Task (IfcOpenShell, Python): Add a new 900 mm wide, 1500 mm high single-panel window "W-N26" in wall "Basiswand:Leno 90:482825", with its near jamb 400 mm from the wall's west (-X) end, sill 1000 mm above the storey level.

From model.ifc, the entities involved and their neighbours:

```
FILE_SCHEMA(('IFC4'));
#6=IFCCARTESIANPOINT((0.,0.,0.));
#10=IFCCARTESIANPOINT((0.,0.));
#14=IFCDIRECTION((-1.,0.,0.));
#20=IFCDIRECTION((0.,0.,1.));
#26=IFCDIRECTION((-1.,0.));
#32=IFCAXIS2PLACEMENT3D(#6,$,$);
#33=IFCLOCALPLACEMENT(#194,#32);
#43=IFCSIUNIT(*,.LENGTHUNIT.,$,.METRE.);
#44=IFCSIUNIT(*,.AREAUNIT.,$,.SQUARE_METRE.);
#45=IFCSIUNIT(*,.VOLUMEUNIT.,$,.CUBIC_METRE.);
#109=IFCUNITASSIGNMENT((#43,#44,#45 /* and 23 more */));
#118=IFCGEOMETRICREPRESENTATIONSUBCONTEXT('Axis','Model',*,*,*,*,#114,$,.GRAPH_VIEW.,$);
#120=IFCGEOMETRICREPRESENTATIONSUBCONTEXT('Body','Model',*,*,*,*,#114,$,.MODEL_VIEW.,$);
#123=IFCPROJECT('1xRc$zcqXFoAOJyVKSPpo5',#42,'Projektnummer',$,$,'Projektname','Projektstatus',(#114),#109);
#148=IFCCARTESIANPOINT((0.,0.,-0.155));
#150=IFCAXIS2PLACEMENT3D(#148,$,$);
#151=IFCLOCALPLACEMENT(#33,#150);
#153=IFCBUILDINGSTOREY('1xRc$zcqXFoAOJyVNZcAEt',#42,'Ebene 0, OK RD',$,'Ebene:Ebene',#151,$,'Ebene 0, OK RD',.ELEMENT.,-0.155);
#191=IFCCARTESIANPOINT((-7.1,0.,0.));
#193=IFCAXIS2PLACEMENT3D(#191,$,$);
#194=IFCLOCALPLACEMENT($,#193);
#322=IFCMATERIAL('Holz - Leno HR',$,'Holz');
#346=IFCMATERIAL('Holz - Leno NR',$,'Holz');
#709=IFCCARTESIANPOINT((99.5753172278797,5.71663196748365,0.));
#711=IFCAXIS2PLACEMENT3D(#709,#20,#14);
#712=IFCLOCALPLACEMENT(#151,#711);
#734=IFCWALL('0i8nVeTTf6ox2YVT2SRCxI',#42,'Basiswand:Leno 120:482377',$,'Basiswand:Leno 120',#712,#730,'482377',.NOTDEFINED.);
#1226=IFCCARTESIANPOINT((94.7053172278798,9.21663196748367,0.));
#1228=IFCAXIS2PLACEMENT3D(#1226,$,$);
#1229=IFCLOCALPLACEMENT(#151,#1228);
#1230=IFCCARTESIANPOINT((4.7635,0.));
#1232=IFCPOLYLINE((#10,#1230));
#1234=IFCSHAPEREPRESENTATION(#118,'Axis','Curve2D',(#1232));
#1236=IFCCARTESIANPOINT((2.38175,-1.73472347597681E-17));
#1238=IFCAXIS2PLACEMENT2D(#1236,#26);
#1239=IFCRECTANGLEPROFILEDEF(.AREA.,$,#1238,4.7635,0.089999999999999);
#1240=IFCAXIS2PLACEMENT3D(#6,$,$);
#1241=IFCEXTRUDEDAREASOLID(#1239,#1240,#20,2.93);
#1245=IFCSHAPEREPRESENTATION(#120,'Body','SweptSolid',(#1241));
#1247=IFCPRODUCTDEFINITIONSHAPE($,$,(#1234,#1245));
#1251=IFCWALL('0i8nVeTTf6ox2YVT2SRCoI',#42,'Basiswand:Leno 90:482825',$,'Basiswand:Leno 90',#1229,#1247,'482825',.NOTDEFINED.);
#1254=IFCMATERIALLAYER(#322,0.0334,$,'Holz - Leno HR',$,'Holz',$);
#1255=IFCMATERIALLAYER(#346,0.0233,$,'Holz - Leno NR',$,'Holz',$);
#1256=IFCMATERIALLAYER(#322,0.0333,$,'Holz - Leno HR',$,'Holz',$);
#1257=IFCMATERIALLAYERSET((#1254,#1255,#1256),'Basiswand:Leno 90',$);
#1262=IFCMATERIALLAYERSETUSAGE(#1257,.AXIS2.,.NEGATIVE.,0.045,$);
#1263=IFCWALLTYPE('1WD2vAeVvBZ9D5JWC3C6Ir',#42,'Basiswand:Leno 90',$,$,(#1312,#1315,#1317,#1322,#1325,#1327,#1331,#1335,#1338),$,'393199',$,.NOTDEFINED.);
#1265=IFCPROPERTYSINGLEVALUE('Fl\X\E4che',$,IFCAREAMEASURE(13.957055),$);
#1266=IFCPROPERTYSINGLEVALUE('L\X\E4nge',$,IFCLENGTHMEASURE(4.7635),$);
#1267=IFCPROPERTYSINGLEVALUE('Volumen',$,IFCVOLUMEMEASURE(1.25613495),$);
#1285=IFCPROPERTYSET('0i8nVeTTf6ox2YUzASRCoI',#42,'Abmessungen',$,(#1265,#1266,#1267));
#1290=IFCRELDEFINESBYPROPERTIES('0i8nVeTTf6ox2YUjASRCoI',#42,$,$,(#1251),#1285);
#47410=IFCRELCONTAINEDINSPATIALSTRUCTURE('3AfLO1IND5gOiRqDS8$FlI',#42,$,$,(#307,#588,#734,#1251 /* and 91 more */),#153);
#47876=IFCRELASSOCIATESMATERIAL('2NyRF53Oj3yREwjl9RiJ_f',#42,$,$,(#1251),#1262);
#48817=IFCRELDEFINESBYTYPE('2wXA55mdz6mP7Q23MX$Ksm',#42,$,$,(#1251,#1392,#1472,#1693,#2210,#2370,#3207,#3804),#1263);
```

```python
import numpy as np
import ifcopenshell
import ifcopenshell.api.feature
import ifcopenshell.api.geometry
import ifcopenshell.api.pset
import ifcopenshell.api.root
import ifcopenshell.api.spatial
import ifcopenshell.geom
import ifcopenshell.util.element
import ifcopenshell.util.placement
import ifcopenshell.util.representation
import ifcopenshell.util.shape
import ifcopenshell.util.unit

model = ifcopenshell.open("model.ifc")
unit_scale = ifcopenshell.util.unit.calculate_unit_scale(model)
area_scale = ifcopenshell.util.unit.calculate_unit_scale(model, "AREAUNIT")
volume_scale = ifcopenshell.util.unit.calculate_unit_scale(model, "VOLUMEUNIT")
settings = ifcopenshell.geom.settings()


def volume(element):
    """Net volume in cubic metres, openings subtracted."""
    shape = ifcopenshell.geom.create_shape(settings, element)
    return ifcopenshell.util.shape.get_volume(shape.geometry)


wall = model.by_guid("0i8nVeTTf6ox2YVT2SRCoI")
storey = ifcopenshell.util.element.get_container(wall, ifc_class="IfcBuildingStorey")
context = ifcopenshell.util.representation.get_context(model, "Model", "Body", "MODEL_VIEW")
before = volume(wall)

width, height, from_end, sill = 0.9, 1.5, 0.4, 1  # metres

# The wall runs along its own X axis, and the end named is its -X end.
wall_shape = ifcopenshell.geom.create_shape(settings, wall)
x, y, z = ifcopenshell.util.shape.get_vertices(wall_shape.geometry).T
start = x.min() + from_end
face, thickness = float(y.min()), float(y.max() - y.min())
wall_matrix = ifcopenshell.util.placement.get_local_placement(wall.ObjectPlacement)
level = ifcopenshell.util.placement.get_local_placement(storey.ObjectPlacement)[2, 3]


def in_wall(x, y):
    """Placement at x, y metres in the wall's axes, at sill height."""
    matrix = wall_matrix.copy()
    matrix[:, 3] = wall_matrix @ np.array([x / unit_scale, y / unit_scale, 0.0, 1.0])
    matrix[2, 3] = level + sill / unit_scale
    return matrix


# Opening: a box that overshoots both wall faces by 50 mm.
opening = ifcopenshell.api.root.create_entity(model, ifc_class="IfcOpeningElement", predefined_type="OPENING")
box = ifcopenshell.api.geometry.add_wall_representation(
    model, context=context, length=width, height=height, thickness=thickness + 0.1
)
ifcopenshell.api.geometry.assign_representation(model, product=opening, representation=box)
ifcopenshell.api.geometry.edit_object_placement(model, product=opening, matrix=in_wall(start, face - 0.05), is_si=False)
ifcopenshell.api.feature.add_feature(model, feature=opening, element=wall)

window = ifcopenshell.api.root.create_entity(model, ifc_class="IfcWindow", name="W-N26", predefined_type="WINDOW")
window.OverallWidth, window.OverallHeight = width / unit_scale, height / unit_scale
window.PartitioningType = "SINGLE_PANEL"
body = ifcopenshell.api.geometry.add_window_representation(
    model,
    context=context,
    overall_width=window.OverallWidth,
    overall_height=window.OverallHeight,
    partition_type="SINGLE_PANEL",
)
ifcopenshell.api.geometry.assign_representation(model, product=window, representation=body)
ifcopenshell.api.spatial.assign_container(model, products=[window], relating_structure=storey)
ifcopenshell.api.feature.add_filling(model, opening=opening, element=window)

# Centre the window in the wall's thickness.
ifcopenshell.api.geometry.edit_object_placement(model, product=window, matrix=in_wall(start, face), is_si=False)
window_shape = ifcopenshell.geom.create_shape(settings, window)
depth = ifcopenshell.util.shape.get_vertices(window_shape.geometry)[:, 1]
offset = face + thickness / 2 - (depth.min() + depth.max()) / 2
ifcopenshell.api.geometry.edit_object_placement(model, product=window, matrix=in_wall(start, offset), is_si=False)

after = volume(wall)

# Update the wall's stored quantities.
pset = model.by_id(ifcopenshell.util.element.get_pset(wall, "Abmessungen", should_inherit=False)["id"])
ifcopenshell.api.pset.edit_pset(model, pset=pset, properties={
    "Fläche": model.create_entity("IfcAreaMeasure", after / thickness / area_scale),
    "Volumen": model.create_entity("IfcVolumeMeasure", after / volume_scale),
})

print(f"wall volume {before:.3f} -> {after:.3f} m3")

model.write("model_edited.ifc")
```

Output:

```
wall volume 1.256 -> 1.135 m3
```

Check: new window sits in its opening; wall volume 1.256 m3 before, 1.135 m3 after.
